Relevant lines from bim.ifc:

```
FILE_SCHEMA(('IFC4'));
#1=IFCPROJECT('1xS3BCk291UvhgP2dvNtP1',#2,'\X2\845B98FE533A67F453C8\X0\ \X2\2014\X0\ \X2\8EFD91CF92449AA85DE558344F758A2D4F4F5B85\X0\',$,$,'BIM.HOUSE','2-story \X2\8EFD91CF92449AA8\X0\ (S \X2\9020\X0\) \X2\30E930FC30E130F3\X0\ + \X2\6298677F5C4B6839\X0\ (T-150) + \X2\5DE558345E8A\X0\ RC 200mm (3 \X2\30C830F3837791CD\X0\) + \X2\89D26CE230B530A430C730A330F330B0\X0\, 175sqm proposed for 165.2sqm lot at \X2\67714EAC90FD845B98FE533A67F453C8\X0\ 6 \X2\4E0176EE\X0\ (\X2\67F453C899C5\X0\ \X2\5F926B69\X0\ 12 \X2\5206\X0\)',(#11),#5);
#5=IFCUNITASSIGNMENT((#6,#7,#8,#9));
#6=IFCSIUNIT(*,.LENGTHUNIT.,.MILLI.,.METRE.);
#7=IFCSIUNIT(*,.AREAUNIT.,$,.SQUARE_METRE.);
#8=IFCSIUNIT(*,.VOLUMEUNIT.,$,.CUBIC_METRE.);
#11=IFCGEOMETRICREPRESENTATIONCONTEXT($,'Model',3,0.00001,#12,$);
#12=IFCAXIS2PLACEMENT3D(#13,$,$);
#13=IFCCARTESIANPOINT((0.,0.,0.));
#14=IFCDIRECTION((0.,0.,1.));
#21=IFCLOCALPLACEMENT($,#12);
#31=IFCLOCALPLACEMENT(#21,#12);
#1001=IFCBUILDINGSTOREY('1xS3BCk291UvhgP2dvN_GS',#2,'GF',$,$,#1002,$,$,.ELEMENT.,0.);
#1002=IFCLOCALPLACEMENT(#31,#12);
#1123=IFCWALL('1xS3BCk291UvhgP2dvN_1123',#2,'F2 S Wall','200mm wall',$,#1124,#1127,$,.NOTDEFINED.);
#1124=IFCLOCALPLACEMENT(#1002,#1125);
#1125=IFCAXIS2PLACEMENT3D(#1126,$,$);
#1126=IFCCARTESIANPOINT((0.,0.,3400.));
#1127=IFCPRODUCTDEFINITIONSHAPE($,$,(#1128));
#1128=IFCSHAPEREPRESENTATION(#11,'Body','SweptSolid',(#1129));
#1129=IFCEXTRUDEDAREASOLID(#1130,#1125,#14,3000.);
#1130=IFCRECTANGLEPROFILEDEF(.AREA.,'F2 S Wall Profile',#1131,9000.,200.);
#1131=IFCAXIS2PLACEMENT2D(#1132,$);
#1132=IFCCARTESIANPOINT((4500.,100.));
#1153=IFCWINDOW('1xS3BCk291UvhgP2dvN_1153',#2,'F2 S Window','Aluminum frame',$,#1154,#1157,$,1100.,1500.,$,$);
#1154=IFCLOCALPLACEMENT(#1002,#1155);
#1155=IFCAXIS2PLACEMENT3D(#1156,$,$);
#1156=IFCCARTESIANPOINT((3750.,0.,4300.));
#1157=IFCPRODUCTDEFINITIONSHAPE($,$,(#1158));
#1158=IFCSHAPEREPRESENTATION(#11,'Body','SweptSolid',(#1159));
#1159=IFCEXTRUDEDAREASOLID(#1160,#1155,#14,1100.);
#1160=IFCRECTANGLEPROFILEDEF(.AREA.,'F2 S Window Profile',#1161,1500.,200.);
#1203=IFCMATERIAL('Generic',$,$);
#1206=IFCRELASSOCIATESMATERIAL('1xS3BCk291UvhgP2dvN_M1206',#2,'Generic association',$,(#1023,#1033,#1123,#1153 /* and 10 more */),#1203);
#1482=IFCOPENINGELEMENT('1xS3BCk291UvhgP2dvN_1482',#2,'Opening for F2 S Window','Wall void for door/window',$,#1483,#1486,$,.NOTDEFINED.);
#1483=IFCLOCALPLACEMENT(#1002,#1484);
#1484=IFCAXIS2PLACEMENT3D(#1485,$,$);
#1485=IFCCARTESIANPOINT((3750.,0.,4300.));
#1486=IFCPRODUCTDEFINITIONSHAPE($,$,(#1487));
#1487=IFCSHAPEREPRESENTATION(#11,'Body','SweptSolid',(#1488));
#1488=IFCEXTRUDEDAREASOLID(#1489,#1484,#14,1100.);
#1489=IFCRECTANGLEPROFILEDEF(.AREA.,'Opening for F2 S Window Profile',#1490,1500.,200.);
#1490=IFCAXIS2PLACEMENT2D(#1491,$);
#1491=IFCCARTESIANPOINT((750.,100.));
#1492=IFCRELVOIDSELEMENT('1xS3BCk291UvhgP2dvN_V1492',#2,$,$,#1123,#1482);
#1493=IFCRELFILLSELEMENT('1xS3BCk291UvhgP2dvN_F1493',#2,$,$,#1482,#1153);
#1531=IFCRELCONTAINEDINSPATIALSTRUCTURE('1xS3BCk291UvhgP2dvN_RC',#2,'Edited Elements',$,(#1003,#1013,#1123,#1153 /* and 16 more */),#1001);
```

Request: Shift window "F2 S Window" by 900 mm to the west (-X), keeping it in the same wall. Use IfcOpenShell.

```python
import ifcopenshell
import ifcopenshell.api.geometry
import ifcopenshell.util.placement

model = ifcopenshell.open("bim.ifc")

window = model.by_id(1153)
opening = window.FillsVoids[0].RelatingOpeningElement
wall = opening.VoidsElements[0].RelatingBuildingElement

wall_matrix = ifcopenshell.util.placement.get_local_placement(wall.ObjectPlacement)
shift = wall_matrix[:3, 0] * -900.0
before = ifcopenshell.util.placement.get_local_placement(window.ObjectPlacement)[:3, 3].copy()

# The window is not placed relative to its opening, so move both.
for product in (opening, window):
    matrix = ifcopenshell.util.placement.get_local_placement(product.ObjectPlacement)
    matrix[:3, 3] += shift
    ifcopenshell.api.geometry.edit_object_placement(model, product=product, matrix=matrix, is_si=False)

after = ifcopenshell.util.placement.get_local_placement(window.ObjectPlacement)[:3, 3]
print("window moved by", (after - before).round(3) + 0.0)

model.write("bim_rev.ifc")
```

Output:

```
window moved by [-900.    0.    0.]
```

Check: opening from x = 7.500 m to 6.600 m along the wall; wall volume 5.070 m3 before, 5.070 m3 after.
